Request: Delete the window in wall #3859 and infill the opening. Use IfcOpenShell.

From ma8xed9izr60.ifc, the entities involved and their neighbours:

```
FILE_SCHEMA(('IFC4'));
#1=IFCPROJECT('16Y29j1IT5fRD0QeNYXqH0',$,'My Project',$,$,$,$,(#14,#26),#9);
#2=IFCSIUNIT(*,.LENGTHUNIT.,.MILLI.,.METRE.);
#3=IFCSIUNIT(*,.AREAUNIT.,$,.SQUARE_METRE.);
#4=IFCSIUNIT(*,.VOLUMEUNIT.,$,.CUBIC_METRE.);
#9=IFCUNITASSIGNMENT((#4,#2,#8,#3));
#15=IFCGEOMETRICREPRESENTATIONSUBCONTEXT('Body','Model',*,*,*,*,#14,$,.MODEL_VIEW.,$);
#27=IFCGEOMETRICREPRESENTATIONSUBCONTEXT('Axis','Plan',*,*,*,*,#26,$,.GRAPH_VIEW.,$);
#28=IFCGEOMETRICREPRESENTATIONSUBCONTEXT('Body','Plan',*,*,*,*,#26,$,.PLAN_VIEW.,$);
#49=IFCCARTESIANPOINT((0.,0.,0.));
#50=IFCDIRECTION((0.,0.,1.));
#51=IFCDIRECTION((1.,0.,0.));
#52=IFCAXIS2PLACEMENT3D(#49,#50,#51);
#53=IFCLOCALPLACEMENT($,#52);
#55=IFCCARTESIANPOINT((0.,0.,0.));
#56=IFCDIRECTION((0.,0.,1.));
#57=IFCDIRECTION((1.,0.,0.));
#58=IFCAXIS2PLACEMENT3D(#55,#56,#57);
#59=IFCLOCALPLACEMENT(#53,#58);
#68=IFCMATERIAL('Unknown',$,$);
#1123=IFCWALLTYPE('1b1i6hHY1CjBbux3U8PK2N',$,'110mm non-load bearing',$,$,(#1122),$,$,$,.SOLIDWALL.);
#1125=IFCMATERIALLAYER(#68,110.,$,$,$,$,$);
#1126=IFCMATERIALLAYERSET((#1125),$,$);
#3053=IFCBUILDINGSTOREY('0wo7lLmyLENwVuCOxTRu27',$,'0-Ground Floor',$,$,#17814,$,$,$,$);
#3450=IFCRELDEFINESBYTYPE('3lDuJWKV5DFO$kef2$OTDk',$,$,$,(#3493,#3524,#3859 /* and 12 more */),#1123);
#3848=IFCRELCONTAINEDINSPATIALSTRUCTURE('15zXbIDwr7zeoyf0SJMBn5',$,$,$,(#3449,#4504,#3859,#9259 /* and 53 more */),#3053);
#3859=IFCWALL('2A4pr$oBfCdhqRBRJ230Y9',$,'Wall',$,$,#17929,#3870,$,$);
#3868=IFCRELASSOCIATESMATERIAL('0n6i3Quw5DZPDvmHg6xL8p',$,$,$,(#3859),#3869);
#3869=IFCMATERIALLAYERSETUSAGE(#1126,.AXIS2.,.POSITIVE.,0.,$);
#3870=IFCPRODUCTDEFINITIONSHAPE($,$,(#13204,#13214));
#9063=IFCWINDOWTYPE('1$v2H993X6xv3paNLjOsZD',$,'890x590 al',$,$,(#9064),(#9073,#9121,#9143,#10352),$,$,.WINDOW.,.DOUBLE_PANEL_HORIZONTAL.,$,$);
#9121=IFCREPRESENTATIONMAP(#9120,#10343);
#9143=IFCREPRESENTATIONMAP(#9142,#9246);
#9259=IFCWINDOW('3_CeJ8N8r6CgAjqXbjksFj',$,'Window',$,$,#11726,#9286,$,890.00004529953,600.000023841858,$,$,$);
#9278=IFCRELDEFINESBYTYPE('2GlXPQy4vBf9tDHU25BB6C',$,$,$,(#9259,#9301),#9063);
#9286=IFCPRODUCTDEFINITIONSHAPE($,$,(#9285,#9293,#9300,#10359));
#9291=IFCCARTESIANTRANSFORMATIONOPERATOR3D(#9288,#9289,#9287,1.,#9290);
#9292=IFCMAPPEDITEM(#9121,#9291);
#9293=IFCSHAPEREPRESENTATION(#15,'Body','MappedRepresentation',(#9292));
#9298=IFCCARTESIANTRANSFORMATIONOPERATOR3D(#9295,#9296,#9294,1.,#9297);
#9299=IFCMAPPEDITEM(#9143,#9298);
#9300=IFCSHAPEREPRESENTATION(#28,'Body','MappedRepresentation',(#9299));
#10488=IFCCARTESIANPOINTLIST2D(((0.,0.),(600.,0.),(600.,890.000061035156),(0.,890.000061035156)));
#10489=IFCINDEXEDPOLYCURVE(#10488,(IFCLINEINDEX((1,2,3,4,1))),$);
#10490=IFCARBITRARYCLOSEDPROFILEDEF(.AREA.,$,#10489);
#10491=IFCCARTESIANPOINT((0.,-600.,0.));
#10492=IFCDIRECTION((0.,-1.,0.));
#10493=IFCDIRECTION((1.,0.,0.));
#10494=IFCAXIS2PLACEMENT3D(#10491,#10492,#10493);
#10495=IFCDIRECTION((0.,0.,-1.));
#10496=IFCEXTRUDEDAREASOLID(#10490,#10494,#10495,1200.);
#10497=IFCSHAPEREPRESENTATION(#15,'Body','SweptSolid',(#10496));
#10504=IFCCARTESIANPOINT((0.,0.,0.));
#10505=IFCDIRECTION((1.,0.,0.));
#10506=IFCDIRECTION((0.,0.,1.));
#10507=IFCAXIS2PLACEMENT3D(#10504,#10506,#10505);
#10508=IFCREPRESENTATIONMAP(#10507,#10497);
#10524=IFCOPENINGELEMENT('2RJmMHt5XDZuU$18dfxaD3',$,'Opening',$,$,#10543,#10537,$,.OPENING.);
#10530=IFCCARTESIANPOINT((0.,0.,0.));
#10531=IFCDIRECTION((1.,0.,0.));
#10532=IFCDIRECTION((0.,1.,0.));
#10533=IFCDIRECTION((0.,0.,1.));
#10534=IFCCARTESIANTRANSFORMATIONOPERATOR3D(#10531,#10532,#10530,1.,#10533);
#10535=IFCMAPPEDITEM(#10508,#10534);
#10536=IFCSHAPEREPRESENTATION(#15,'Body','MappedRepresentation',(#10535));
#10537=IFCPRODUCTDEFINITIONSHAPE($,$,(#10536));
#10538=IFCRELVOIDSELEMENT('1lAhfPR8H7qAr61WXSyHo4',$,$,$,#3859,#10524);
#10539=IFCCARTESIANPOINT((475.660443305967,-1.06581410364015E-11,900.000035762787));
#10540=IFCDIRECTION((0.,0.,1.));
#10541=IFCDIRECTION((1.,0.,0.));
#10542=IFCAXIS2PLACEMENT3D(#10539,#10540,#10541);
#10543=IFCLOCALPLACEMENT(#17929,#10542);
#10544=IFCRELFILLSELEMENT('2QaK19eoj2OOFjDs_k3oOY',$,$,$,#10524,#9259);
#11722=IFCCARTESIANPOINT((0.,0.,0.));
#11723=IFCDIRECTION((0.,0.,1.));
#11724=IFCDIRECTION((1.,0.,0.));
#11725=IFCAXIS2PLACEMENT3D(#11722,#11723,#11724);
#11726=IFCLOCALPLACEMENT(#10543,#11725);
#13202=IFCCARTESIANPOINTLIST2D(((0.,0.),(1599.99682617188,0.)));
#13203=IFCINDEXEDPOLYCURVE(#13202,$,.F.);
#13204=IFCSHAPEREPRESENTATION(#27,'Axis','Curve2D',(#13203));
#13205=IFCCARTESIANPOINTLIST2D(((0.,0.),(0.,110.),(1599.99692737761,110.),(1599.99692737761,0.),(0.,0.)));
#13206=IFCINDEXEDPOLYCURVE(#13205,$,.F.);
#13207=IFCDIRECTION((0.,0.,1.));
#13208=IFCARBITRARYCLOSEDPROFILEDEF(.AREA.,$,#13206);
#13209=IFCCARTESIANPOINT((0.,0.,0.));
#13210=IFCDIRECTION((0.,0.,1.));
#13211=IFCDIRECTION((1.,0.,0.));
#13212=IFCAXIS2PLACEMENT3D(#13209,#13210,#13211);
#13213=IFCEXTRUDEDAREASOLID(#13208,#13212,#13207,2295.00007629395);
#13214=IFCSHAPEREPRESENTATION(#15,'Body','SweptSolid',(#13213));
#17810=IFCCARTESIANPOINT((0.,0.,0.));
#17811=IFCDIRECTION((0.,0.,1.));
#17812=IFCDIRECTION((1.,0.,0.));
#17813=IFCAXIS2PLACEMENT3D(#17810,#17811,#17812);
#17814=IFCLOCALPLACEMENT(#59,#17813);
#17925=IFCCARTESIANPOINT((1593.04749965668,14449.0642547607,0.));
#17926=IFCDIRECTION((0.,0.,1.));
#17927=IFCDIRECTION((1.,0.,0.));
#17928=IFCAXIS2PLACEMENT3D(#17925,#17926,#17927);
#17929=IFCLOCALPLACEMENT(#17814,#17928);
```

```python
import ifcopenshell
import ifcopenshell.api.feature
import ifcopenshell.api.root
import ifcopenshell.geom
import ifcopenshell.util.shape

model = ifcopenshell.open("ma8xed9izr60.ifc")
settings = ifcopenshell.geom.settings()


def volume(element):
    """Net volume in cubic metres, openings subtracted."""
    shape = ifcopenshell.geom.create_shape(settings, element)
    return ifcopenshell.util.shape.get_volume(shape.geometry)


window = model.by_guid("3_CeJ8N8r6CgAjqXbjksFj")
opening = window.FillsVoids[0].RelatingOpeningElement
wall = opening.VoidsElements[0].RelatingBuildingElement
before = volume(wall)

ifcopenshell.api.root.remove_product(model, product=window)
ifcopenshell.api.feature.remove_feature(model, feature=opening)

after = volume(wall)

print(f"wall volume {before:.3f} -> {after:.3f} m3")

model.write("ma8xed9izr60-out.ifc")
```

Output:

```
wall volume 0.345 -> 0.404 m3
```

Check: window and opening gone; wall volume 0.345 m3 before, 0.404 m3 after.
